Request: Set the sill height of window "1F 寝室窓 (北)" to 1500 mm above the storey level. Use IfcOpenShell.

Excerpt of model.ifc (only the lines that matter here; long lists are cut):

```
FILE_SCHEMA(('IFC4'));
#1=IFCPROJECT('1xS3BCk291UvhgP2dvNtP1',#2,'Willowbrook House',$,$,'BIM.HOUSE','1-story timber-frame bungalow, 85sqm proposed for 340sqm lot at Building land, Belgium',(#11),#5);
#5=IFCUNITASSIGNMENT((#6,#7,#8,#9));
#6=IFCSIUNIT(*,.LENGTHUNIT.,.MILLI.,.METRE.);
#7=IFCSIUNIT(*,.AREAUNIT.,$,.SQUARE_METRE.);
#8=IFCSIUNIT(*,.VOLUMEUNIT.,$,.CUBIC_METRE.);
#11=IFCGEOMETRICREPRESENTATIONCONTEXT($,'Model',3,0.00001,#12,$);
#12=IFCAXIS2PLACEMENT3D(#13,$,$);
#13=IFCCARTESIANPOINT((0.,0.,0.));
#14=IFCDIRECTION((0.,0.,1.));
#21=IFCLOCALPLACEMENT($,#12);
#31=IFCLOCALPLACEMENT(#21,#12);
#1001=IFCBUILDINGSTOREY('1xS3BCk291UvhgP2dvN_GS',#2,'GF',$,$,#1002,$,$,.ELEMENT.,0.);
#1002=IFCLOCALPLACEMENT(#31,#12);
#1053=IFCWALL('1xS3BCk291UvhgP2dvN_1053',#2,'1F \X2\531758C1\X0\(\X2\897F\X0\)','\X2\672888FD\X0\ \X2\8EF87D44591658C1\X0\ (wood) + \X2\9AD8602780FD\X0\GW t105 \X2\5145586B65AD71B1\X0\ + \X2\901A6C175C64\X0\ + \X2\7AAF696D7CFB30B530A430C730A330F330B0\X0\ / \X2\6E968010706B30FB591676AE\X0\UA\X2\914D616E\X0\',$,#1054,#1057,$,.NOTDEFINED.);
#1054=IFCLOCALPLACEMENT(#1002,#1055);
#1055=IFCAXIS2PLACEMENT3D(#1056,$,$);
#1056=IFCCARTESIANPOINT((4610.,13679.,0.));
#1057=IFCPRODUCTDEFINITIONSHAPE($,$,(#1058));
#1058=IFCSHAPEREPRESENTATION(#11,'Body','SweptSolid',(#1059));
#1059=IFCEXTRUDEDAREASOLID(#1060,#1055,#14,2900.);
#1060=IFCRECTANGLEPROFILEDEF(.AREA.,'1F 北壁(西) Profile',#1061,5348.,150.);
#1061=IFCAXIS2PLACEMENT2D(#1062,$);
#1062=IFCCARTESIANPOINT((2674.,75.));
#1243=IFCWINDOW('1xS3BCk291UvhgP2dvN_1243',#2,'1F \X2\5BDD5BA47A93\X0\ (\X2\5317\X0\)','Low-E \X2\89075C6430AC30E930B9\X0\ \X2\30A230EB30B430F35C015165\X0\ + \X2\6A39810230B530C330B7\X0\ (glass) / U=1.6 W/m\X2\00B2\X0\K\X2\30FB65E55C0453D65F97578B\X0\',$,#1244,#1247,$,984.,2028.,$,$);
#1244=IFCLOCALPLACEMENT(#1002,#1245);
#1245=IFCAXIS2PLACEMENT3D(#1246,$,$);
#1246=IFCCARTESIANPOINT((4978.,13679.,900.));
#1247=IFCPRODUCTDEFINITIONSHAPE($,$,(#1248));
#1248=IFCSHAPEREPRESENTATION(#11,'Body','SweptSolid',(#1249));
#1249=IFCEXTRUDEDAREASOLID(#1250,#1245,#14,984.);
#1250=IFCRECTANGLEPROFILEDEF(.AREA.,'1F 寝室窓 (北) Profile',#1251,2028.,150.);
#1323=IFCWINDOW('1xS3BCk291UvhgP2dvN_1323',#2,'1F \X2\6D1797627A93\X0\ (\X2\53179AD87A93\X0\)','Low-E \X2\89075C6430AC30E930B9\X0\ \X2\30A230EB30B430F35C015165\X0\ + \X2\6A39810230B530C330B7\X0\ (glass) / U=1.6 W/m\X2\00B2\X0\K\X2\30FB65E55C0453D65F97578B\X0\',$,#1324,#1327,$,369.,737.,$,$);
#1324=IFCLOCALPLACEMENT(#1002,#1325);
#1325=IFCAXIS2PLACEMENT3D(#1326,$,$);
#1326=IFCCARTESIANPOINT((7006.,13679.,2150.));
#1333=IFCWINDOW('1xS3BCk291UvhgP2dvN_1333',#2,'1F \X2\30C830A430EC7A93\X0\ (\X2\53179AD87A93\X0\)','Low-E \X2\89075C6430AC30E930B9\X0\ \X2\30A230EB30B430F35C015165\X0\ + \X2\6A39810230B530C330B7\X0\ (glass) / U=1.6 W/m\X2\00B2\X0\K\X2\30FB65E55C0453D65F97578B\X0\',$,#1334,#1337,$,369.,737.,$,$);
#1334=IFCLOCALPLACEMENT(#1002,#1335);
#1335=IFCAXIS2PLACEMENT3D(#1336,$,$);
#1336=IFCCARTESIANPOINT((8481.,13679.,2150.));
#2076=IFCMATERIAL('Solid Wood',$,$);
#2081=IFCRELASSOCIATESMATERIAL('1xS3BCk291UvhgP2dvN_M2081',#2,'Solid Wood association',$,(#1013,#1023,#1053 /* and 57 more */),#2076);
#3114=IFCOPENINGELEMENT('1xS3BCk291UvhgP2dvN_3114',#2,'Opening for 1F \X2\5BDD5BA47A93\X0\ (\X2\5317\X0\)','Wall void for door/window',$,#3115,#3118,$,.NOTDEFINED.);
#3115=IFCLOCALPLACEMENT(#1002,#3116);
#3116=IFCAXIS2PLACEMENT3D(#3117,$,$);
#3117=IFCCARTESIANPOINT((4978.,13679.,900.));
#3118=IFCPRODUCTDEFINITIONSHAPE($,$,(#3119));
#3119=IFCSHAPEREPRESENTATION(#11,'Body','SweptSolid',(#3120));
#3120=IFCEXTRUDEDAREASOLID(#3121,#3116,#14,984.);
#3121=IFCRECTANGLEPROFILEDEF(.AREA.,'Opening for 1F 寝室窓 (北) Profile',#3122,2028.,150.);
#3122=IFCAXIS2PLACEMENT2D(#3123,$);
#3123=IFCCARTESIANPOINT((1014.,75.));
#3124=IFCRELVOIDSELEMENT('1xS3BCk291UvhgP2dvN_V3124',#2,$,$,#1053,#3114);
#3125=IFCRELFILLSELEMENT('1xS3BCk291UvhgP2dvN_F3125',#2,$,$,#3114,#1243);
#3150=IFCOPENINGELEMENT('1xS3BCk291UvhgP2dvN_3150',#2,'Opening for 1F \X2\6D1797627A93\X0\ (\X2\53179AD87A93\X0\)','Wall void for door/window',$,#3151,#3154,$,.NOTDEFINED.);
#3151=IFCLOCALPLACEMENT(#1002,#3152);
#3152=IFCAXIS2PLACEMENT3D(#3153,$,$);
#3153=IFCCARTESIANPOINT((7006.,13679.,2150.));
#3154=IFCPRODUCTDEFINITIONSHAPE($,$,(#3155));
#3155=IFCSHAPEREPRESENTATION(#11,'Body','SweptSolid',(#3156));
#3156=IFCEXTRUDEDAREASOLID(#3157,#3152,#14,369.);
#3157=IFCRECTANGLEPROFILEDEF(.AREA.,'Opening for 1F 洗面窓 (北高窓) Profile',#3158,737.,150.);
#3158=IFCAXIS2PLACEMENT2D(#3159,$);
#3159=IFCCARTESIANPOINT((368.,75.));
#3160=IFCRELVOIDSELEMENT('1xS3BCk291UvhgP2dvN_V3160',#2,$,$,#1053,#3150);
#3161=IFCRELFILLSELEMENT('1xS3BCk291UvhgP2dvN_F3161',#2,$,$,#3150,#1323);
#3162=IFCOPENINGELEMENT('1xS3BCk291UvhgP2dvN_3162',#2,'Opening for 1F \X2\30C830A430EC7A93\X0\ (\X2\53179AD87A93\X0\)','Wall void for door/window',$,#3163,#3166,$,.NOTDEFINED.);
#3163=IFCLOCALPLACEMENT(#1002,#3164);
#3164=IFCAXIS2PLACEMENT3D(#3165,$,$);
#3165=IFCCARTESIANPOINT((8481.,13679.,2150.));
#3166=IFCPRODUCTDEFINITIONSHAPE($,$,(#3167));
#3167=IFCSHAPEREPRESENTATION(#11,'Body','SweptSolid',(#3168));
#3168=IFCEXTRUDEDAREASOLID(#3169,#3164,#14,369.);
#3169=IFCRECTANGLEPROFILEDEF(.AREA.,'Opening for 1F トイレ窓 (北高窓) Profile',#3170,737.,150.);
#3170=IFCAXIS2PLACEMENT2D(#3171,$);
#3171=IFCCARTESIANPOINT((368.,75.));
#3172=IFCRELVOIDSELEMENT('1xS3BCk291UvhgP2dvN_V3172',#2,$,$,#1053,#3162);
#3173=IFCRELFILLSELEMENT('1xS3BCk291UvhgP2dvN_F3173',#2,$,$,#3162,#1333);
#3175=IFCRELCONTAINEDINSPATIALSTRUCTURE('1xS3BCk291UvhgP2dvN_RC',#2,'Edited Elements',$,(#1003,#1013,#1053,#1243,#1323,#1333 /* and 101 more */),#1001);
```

```python
import numpy as np
import ifcopenshell
import ifcopenshell.api.geometry
import ifcopenshell.geom
import ifcopenshell.util.element
import ifcopenshell.util.placement
import ifcopenshell.util.shape
import ifcopenshell.util.unit

model = ifcopenshell.open("model.ifc")
unit_scale = ifcopenshell.util.unit.calculate_unit_scale(model)

window = model.by_guid("1xS3BCk291UvhgP2dvN_1243")
opening = window.FillsVoids[0].RelatingOpeningElement
storey = ifcopenshell.util.element.get_container(window, ifc_class="IfcBuildingStorey")
level = ifcopenshell.util.placement.get_local_placement(storey.ObjectPlacement)[2, 3]

# The opening's origin need not be at the sill, so measure its lowest point.
shape = ifcopenshell.geom.create_shape(ifcopenshell.geom.settings(), opening)
bottom = ifcopenshell.util.shape.get_shape_bottom_elevation(shape, shape.geometry) / unit_scale
dz = level + 1500.0 - bottom

shift = np.array([0.0, 0.0, dz])
# The window is not placed relative to its opening, so move both.
for product in (opening, window):
    matrix = ifcopenshell.util.placement.get_local_placement(product.ObjectPlacement)
    matrix[:3, 3] += shift
    ifcopenshell.api.geometry.edit_object_placement(model, product=product, matrix=matrix, is_si=False)

print(f"moved by {dz * unit_scale:+.3f} m")

model.write("model_edited.ifc")
```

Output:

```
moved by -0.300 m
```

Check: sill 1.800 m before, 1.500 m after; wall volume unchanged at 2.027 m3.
